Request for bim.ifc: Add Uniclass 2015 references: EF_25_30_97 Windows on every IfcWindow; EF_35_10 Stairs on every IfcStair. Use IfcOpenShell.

First a look at what the model holds.

```python
import ifcopenshell

model = ifcopenshell.open("bim.ifc")
print(model.schema)
print("classifications:", [c.Name for c in model.by_type("IfcClassification")])
for ifc_class in ("IfcDoor", "IfcRoof", "IfcStair", "IfcWall", "IfcWindow"):
    print(ifc_class, len(model.by_type(ifc_class)))
```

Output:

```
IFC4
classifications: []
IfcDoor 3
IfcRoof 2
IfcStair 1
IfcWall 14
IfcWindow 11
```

```python
import ifcopenshell
import ifcopenshell.api.classification

model = ifcopenshell.open("bim.ifc")

system = ifcopenshell.api.classification.add_classification(model, classification="Uniclass 2015")

codes = {
    "IfcWindow": ("EF_25_30_97", "Windows"),
    "IfcStair": ("EF_35_10", "Stairs"),
}
for ifc_class, (code, name) in codes.items():
    products = model.by_type(ifc_class)
    ifcopenshell.api.classification.add_reference(
        model, products=products, classification=system, identification=code, name=name
    )
    print(code, len(products))

model.write("bim_rev.ifc")
```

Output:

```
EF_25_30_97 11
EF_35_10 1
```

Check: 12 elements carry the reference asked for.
